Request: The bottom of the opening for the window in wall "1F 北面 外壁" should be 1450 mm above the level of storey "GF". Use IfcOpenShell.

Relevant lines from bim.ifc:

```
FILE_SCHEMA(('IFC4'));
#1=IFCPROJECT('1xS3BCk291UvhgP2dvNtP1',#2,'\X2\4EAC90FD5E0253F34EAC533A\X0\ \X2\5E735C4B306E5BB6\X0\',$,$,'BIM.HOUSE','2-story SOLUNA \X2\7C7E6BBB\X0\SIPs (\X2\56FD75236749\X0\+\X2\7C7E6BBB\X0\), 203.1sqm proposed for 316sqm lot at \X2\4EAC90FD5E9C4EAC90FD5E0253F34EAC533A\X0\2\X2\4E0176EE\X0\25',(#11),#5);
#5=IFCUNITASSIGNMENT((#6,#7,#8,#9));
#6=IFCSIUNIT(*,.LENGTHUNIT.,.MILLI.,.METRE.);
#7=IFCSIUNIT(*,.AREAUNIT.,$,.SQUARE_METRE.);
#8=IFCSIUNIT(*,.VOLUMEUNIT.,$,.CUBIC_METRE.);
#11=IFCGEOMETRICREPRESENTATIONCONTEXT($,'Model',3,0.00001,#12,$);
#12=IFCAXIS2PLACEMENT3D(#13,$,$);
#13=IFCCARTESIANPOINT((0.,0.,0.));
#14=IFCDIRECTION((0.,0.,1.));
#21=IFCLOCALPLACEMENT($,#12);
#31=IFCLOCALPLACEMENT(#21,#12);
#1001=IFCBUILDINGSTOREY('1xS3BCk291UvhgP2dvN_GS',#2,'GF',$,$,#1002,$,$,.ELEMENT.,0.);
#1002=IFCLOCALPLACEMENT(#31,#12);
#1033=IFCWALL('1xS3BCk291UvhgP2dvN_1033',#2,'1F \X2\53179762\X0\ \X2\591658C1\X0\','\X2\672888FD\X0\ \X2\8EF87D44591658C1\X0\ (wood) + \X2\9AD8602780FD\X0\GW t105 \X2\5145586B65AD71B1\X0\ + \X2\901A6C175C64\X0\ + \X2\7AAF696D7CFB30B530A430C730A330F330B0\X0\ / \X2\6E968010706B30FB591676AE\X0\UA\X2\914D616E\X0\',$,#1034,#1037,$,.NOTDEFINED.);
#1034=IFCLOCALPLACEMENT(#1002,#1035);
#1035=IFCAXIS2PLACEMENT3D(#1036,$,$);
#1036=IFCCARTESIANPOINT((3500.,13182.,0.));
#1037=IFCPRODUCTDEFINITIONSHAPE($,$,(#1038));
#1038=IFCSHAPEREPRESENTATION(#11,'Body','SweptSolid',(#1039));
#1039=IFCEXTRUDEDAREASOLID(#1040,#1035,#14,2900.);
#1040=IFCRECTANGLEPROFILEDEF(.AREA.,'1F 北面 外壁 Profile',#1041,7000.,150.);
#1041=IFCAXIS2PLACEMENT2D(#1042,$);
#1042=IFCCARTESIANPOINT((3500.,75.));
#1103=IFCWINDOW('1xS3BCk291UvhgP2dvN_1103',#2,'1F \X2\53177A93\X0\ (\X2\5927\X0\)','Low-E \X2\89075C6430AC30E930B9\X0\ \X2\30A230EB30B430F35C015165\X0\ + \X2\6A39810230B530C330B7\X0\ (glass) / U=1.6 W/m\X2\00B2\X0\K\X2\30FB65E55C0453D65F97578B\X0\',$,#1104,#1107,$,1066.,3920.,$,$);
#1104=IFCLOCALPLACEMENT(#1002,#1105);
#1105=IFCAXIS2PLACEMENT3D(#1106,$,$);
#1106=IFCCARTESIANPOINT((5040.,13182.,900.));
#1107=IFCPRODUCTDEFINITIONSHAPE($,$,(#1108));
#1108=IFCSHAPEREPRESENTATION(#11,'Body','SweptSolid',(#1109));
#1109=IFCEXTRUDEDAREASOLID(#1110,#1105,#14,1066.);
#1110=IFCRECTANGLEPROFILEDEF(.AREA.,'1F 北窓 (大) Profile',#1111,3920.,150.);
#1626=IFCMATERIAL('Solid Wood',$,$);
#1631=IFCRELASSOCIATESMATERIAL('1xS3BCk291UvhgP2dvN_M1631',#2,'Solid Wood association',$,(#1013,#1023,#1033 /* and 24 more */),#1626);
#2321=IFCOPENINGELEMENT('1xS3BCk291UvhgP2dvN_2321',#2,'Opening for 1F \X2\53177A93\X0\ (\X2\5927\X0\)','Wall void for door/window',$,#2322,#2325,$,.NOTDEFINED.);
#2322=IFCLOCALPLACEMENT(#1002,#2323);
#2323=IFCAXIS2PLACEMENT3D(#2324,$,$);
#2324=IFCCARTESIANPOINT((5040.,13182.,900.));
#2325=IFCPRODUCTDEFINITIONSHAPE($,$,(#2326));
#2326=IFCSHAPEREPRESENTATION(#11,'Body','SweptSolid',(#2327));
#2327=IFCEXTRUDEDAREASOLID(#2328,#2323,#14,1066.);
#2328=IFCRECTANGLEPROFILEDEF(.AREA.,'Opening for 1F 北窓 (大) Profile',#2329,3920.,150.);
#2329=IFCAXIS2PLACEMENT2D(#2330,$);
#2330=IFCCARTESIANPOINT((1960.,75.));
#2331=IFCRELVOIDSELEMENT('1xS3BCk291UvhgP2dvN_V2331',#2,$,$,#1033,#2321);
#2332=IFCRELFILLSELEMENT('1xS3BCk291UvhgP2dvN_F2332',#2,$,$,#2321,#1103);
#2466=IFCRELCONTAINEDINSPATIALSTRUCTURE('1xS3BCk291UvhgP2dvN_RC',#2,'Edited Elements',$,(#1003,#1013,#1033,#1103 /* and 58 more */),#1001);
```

```python
import numpy as np
import ifcopenshell
import ifcopenshell.api.geometry
import ifcopenshell.geom
import ifcopenshell.util.element
import ifcopenshell.util.placement
import ifcopenshell.util.shape
import ifcopenshell.util.unit

model = ifcopenshell.open("bim.ifc")
unit_scale = ifcopenshell.util.unit.calculate_unit_scale(model)

window = model.by_guid("1xS3BCk291UvhgP2dvN_1103")
opening = window.FillsVoids[0].RelatingOpeningElement
storey = ifcopenshell.util.element.get_container(window, ifc_class="IfcBuildingStorey")
level = ifcopenshell.util.placement.get_local_placement(storey.ObjectPlacement)[2, 3]

# The opening's origin need not be at the sill, so measure its lowest point.
shape = ifcopenshell.geom.create_shape(ifcopenshell.geom.settings(), opening)
bottom = ifcopenshell.util.shape.get_shape_bottom_elevation(shape, shape.geometry) / unit_scale
dz = level + 1450.0 - bottom

shift = np.array([0.0, 0.0, dz])
# The window is not placed relative to its opening, so move both.
for product in (opening, window):
    matrix = ifcopenshell.util.placement.get_local_placement(product.ObjectPlacement)
    matrix[:3, 3] += shift
    ifcopenshell.api.geometry.edit_object_placement(model, product=product, matrix=matrix, is_si=False)

print(f"moved by {dz * unit_scale:+.3f} m")

model.write("bim_rev.ifc")
```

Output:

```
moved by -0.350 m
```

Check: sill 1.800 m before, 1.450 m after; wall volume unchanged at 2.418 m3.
